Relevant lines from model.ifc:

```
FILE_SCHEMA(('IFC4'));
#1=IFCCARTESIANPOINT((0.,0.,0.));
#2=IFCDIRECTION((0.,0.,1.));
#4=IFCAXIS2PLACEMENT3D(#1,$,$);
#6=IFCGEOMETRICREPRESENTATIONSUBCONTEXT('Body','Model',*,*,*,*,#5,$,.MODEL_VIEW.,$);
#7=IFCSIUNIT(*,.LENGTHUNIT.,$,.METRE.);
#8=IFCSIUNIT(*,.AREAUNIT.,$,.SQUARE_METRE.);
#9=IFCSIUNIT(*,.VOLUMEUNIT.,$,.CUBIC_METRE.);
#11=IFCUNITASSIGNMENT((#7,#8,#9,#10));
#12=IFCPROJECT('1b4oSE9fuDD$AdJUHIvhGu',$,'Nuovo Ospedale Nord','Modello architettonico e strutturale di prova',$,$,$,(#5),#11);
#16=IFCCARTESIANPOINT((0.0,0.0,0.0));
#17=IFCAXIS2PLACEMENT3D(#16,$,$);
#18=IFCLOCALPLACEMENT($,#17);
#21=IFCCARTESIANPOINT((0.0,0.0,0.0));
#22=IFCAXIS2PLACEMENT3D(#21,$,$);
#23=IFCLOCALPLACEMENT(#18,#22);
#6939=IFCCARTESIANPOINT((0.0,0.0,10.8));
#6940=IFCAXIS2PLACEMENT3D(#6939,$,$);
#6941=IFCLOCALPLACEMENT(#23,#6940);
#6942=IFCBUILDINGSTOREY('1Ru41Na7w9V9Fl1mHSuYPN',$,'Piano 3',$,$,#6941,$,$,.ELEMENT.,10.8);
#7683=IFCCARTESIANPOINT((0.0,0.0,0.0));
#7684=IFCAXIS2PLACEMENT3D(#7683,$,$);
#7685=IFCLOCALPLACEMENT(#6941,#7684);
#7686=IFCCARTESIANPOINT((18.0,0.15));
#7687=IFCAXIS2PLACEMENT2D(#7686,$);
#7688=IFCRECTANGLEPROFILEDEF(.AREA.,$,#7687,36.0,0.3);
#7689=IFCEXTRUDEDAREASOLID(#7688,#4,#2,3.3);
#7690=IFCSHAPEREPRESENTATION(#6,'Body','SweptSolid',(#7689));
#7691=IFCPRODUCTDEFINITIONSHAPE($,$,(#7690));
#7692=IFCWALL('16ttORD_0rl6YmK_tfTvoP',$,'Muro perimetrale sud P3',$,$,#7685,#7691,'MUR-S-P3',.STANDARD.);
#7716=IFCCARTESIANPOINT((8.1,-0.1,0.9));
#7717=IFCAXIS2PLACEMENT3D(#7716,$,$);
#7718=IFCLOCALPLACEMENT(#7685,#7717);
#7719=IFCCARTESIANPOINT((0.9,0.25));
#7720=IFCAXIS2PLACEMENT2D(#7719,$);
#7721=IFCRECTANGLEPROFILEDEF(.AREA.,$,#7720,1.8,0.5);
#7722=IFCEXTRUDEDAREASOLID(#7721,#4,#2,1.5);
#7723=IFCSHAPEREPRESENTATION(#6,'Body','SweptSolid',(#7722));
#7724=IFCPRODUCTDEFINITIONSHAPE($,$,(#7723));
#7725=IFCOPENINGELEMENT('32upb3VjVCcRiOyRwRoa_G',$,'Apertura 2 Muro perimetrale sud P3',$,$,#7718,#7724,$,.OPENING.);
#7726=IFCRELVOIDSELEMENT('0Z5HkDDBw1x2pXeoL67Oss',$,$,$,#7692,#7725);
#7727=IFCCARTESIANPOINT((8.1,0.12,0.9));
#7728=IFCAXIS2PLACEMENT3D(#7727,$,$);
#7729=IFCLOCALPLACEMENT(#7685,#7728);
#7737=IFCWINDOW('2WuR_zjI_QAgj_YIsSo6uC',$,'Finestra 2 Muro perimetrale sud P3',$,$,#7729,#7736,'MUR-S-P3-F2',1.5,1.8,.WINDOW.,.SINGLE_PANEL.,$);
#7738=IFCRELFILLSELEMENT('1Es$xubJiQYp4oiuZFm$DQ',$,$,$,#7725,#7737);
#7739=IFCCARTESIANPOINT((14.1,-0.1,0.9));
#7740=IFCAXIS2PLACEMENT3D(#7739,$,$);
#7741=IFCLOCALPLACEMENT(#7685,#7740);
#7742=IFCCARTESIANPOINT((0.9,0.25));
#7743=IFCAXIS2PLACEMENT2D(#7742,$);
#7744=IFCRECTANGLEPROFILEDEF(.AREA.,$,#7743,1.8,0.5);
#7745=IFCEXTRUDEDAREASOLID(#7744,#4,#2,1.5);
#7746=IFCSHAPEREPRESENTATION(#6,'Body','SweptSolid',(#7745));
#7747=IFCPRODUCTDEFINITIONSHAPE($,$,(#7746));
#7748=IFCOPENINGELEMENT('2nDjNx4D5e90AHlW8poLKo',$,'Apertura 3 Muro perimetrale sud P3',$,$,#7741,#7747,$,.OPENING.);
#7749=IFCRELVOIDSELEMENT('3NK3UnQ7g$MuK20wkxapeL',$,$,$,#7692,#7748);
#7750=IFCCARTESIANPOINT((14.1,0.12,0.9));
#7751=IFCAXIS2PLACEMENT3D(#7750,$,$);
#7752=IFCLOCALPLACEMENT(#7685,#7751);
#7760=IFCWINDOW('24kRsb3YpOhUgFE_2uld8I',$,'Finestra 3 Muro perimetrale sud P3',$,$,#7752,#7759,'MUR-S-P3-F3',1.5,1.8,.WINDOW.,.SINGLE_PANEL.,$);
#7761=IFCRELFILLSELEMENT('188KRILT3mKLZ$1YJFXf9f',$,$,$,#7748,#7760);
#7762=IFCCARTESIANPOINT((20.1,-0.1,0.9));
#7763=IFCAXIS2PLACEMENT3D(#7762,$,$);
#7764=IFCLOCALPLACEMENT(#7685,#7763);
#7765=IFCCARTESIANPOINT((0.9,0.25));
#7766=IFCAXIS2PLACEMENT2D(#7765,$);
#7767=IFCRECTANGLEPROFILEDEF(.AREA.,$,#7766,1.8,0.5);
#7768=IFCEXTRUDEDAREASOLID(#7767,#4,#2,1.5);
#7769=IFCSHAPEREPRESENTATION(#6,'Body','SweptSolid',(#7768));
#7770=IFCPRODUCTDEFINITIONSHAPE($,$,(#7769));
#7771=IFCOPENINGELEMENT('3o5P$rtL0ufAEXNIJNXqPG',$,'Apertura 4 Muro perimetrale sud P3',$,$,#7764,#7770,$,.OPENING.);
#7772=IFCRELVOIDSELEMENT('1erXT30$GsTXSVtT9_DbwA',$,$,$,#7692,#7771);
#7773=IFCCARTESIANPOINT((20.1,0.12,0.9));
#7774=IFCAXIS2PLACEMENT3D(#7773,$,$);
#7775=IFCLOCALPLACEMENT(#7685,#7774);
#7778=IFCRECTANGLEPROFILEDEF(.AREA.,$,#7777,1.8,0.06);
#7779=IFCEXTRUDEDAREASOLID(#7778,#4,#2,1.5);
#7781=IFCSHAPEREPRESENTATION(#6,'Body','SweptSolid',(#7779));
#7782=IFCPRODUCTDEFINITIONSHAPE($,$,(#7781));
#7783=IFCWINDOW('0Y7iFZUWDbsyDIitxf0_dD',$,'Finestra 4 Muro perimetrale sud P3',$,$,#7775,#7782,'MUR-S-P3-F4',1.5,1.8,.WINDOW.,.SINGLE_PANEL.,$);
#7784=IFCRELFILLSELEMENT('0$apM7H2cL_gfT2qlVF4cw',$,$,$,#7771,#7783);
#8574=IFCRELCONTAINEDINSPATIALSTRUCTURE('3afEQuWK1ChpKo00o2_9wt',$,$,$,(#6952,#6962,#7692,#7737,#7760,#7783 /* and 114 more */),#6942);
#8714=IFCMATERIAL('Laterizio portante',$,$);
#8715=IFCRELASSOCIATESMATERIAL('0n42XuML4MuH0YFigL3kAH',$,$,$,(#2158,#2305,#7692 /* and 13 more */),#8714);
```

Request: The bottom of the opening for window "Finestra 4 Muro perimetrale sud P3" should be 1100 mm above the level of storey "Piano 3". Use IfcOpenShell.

```python
import numpy as np
import ifcopenshell
import ifcopenshell.api.geometry
import ifcopenshell.geom
import ifcopenshell.util.element
import ifcopenshell.util.placement
import ifcopenshell.util.shape
import ifcopenshell.util.unit

model = ifcopenshell.open("model.ifc")
unit_scale = ifcopenshell.util.unit.calculate_unit_scale(model)

window = model.by_id(7783)
opening = window.FillsVoids[0].RelatingOpeningElement
storey = ifcopenshell.util.element.get_container(window, ifc_class="IfcBuildingStorey")
level = ifcopenshell.util.placement.get_local_placement(storey.ObjectPlacement)[2, 3]

# The opening's origin need not be at the sill, so measure its lowest point.
shape = ifcopenshell.geom.create_shape(ifcopenshell.geom.settings(), opening)
bottom = ifcopenshell.util.shape.get_shape_bottom_elevation(shape, shape.geometry) / unit_scale
dz = level + 1.1 / unit_scale - bottom

shift = np.array([0.0, 0.0, dz])
# The window is not placed relative to its opening, so move both.
for product in (opening, window):
    matrix = ifcopenshell.util.placement.get_local_placement(product.ObjectPlacement)
    matrix[:3, 3] += shift
    ifcopenshell.api.geometry.edit_object_placement(model, product=product, matrix=matrix, is_si=False)

print(f"moved by {dz * unit_scale:+.3f} m")

model.write("model-out.ifc")
```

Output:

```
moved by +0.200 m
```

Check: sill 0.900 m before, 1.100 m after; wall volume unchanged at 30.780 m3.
